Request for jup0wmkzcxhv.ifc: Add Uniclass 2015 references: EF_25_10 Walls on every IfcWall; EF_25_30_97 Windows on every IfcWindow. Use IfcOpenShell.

First a look at what the model holds.

```python
import ifcopenshell

model = ifcopenshell.open("jup0wmkzcxhv.ifc")
print(model.schema)
print("classifications:", [c.Name for c in model.by_type("IfcClassification")])
for ifc_class in ("IfcDoor", "IfcRoof", "IfcStair", "IfcWall", "IfcWindow"):
    print(ifc_class, len(model.by_type(ifc_class)))
```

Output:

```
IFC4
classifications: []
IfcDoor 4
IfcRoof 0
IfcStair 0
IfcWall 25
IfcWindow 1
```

```python
import ifcopenshell
import ifcopenshell.api.classification

model = ifcopenshell.open("jup0wmkzcxhv.ifc")

system = ifcopenshell.api.classification.add_classification(model, classification="Uniclass 2015")

codes = {
    "IfcWall": ("EF_25_10", "Walls"),
    "IfcWindow": ("EF_25_30_97", "Windows"),
}
for ifc_class, (code, name) in codes.items():
    products = model.by_type(ifc_class)
    ifcopenshell.api.classification.add_reference(
        model, products=products, classification=system, identification=code, name=name
    )
    print(code, len(products))

model.write("jup0wmkzcxhv_rev.ifc")
```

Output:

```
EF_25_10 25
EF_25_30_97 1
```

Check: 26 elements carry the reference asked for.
